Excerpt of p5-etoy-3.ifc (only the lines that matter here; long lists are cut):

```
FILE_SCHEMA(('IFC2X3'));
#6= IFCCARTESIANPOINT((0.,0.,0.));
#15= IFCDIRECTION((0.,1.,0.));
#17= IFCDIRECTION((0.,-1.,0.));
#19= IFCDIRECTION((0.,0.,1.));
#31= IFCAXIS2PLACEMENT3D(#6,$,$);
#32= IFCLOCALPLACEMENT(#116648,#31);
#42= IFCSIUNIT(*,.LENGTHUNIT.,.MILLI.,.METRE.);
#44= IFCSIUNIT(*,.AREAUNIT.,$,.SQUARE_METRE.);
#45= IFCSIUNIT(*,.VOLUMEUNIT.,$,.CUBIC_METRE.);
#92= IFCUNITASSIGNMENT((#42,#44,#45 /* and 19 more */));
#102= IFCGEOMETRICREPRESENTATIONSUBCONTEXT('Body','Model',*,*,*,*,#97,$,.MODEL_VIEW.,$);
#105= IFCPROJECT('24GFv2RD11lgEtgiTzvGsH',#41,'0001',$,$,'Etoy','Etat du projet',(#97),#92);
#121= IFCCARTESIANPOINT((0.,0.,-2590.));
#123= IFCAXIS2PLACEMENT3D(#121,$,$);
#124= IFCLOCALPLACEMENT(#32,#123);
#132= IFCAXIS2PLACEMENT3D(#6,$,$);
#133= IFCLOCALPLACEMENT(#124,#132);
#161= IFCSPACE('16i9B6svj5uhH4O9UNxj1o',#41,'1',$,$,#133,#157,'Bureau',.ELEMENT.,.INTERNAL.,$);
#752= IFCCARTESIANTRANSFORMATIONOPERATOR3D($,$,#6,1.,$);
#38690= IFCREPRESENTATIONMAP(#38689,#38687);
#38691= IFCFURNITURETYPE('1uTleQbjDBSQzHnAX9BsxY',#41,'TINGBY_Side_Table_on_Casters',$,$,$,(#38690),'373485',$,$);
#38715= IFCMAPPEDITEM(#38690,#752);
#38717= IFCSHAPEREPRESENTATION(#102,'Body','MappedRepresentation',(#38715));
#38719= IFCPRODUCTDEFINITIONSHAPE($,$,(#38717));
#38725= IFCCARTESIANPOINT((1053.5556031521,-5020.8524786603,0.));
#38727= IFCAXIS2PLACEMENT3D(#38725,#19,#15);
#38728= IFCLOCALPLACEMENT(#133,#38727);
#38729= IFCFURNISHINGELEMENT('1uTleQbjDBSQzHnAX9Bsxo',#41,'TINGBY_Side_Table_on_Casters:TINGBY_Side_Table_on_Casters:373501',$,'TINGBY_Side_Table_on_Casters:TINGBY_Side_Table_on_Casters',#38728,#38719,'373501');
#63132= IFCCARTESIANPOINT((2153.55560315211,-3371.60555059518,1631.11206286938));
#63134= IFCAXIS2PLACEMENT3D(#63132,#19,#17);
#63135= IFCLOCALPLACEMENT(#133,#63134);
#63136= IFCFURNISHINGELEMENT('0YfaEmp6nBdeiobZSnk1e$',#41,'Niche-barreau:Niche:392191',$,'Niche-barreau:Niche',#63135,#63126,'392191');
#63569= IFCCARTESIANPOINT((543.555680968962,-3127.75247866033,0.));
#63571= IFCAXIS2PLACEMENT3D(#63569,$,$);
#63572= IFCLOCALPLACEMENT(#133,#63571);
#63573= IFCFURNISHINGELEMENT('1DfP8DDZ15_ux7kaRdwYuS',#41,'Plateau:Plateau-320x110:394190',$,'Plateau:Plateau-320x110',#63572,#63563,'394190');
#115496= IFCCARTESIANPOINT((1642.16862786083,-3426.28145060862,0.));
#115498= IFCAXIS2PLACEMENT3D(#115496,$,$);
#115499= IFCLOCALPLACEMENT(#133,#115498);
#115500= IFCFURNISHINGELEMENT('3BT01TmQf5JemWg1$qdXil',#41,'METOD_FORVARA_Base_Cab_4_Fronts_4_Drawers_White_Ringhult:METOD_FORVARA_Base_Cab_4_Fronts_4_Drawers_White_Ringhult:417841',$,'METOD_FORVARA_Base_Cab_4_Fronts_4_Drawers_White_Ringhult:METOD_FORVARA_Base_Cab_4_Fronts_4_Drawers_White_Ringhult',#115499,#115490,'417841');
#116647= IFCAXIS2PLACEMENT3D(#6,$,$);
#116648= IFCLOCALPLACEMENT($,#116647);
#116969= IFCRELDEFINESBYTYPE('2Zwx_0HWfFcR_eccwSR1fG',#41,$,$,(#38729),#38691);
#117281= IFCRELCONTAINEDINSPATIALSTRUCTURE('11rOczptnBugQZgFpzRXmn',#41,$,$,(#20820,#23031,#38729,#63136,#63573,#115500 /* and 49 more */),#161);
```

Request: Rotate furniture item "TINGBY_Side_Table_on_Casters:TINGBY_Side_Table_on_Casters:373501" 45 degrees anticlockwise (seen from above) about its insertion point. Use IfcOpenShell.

```python
import ifcopenshell
import ifcopenshell.api.geometry
import ifcopenshell.util.placement

model = ifcopenshell.open("p5-etoy-3.ifc")

item = model.by_guid("1uTleQbjDBSQzHnAX9Bsxo")
matrix = ifcopenshell.util.placement.get_local_placement(item.ObjectPlacement)
matrix = matrix @ ifcopenshell.util.placement.rotation(45, "Z")
ifcopenshell.api.geometry.edit_object_placement(model, product=item, matrix=matrix, is_si=False)

print(ifcopenshell.util.placement.get_local_placement(item.ObjectPlacement).round(3) + 0.0)

model.write("p5-etoy-3_v2.ifc")
```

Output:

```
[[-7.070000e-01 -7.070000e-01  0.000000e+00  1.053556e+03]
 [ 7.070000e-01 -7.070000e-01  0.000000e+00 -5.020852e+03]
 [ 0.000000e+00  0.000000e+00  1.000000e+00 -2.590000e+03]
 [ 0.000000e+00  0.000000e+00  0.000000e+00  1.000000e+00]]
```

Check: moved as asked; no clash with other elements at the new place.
